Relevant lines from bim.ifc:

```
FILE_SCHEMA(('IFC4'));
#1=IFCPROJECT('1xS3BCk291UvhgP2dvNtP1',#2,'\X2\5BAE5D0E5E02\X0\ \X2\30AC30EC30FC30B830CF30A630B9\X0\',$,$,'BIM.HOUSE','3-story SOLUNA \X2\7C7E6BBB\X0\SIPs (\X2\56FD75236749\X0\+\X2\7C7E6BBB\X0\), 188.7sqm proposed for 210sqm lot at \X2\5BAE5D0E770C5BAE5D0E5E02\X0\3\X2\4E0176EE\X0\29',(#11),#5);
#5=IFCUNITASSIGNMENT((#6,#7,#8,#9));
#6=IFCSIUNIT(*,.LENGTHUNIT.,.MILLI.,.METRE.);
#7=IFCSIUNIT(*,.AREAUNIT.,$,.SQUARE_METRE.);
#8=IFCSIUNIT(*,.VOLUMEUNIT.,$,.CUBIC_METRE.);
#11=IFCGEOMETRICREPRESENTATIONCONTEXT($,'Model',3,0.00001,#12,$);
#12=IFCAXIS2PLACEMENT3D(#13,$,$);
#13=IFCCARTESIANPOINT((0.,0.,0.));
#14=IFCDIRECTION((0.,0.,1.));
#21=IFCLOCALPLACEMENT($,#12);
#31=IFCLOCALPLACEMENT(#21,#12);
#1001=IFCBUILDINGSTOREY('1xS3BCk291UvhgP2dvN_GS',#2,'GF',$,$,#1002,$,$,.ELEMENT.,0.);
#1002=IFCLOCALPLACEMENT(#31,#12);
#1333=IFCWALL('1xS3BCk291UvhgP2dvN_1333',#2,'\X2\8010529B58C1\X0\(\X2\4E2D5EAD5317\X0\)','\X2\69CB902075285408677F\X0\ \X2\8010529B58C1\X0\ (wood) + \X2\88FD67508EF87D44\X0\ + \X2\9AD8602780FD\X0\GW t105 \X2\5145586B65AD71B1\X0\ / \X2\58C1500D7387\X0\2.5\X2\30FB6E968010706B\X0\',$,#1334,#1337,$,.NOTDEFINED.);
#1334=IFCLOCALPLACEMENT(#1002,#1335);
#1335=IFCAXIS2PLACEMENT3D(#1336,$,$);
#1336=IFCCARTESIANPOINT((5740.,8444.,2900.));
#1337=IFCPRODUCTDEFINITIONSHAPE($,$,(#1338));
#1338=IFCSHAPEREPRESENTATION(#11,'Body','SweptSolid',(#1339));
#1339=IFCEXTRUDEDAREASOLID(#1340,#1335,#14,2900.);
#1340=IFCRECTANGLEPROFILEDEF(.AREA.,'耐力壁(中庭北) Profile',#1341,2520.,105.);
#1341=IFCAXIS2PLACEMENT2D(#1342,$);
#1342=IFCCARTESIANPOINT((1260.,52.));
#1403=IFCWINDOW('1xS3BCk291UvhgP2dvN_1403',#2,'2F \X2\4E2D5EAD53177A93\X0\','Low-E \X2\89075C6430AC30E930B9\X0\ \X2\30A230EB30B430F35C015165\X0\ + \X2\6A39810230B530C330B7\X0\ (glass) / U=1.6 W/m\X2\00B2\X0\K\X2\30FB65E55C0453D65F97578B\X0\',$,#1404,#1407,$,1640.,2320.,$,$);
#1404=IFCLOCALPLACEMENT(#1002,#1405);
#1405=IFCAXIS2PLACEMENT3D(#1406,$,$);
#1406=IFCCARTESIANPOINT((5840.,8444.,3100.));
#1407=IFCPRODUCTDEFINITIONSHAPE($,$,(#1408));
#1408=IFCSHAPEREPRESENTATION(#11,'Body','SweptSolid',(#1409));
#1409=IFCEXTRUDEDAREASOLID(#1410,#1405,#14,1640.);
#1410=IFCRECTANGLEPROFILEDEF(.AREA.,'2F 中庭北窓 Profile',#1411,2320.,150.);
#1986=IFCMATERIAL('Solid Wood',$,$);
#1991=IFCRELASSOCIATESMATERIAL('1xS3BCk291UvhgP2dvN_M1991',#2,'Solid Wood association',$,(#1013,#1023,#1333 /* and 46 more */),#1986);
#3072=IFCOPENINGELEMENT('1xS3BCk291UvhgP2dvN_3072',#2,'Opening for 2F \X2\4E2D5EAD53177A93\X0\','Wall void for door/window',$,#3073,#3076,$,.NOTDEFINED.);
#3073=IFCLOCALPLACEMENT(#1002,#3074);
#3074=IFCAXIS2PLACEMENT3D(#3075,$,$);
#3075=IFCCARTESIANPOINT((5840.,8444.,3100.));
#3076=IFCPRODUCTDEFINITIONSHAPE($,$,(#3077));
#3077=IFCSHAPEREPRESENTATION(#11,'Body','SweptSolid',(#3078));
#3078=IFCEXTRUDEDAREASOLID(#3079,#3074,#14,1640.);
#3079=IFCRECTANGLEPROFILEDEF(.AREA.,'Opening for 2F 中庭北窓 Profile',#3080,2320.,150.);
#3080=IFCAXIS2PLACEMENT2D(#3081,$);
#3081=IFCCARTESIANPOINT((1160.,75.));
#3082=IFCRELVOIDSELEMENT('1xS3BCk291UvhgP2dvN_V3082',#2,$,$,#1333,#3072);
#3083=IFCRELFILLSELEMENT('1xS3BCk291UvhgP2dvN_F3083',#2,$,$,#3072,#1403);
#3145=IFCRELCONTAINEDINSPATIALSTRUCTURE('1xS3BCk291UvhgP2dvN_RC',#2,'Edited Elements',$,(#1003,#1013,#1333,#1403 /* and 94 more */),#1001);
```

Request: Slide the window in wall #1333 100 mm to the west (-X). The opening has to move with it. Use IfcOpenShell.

```python
import ifcopenshell
import ifcopenshell.api.geometry
import ifcopenshell.util.placement

model = ifcopenshell.open("bim.ifc")

window = model.by_id(1403)
opening = window.FillsVoids[0].RelatingOpeningElement
wall = opening.VoidsElements[0].RelatingBuildingElement

wall_matrix = ifcopenshell.util.placement.get_local_placement(wall.ObjectPlacement)
shift = wall_matrix[:3, 0] * -100.0
before = ifcopenshell.util.placement.get_local_placement(window.ObjectPlacement)[:3, 3].copy()

# The window is not placed relative to its opening, so move both.
for product in (opening, window):
    matrix = ifcopenshell.util.placement.get_local_placement(product.ObjectPlacement)
    matrix[:3, 3] += shift
    ifcopenshell.api.geometry.edit_object_placement(model, product=product, matrix=matrix, is_si=False)

after = ifcopenshell.util.placement.get_local_placement(window.ObjectPlacement)[:3, 3]
print("window moved by", (after - before).round(3) + 0.0)

model.write("bim-out.ifc")
```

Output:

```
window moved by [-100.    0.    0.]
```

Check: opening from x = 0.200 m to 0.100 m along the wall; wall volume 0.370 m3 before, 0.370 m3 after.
